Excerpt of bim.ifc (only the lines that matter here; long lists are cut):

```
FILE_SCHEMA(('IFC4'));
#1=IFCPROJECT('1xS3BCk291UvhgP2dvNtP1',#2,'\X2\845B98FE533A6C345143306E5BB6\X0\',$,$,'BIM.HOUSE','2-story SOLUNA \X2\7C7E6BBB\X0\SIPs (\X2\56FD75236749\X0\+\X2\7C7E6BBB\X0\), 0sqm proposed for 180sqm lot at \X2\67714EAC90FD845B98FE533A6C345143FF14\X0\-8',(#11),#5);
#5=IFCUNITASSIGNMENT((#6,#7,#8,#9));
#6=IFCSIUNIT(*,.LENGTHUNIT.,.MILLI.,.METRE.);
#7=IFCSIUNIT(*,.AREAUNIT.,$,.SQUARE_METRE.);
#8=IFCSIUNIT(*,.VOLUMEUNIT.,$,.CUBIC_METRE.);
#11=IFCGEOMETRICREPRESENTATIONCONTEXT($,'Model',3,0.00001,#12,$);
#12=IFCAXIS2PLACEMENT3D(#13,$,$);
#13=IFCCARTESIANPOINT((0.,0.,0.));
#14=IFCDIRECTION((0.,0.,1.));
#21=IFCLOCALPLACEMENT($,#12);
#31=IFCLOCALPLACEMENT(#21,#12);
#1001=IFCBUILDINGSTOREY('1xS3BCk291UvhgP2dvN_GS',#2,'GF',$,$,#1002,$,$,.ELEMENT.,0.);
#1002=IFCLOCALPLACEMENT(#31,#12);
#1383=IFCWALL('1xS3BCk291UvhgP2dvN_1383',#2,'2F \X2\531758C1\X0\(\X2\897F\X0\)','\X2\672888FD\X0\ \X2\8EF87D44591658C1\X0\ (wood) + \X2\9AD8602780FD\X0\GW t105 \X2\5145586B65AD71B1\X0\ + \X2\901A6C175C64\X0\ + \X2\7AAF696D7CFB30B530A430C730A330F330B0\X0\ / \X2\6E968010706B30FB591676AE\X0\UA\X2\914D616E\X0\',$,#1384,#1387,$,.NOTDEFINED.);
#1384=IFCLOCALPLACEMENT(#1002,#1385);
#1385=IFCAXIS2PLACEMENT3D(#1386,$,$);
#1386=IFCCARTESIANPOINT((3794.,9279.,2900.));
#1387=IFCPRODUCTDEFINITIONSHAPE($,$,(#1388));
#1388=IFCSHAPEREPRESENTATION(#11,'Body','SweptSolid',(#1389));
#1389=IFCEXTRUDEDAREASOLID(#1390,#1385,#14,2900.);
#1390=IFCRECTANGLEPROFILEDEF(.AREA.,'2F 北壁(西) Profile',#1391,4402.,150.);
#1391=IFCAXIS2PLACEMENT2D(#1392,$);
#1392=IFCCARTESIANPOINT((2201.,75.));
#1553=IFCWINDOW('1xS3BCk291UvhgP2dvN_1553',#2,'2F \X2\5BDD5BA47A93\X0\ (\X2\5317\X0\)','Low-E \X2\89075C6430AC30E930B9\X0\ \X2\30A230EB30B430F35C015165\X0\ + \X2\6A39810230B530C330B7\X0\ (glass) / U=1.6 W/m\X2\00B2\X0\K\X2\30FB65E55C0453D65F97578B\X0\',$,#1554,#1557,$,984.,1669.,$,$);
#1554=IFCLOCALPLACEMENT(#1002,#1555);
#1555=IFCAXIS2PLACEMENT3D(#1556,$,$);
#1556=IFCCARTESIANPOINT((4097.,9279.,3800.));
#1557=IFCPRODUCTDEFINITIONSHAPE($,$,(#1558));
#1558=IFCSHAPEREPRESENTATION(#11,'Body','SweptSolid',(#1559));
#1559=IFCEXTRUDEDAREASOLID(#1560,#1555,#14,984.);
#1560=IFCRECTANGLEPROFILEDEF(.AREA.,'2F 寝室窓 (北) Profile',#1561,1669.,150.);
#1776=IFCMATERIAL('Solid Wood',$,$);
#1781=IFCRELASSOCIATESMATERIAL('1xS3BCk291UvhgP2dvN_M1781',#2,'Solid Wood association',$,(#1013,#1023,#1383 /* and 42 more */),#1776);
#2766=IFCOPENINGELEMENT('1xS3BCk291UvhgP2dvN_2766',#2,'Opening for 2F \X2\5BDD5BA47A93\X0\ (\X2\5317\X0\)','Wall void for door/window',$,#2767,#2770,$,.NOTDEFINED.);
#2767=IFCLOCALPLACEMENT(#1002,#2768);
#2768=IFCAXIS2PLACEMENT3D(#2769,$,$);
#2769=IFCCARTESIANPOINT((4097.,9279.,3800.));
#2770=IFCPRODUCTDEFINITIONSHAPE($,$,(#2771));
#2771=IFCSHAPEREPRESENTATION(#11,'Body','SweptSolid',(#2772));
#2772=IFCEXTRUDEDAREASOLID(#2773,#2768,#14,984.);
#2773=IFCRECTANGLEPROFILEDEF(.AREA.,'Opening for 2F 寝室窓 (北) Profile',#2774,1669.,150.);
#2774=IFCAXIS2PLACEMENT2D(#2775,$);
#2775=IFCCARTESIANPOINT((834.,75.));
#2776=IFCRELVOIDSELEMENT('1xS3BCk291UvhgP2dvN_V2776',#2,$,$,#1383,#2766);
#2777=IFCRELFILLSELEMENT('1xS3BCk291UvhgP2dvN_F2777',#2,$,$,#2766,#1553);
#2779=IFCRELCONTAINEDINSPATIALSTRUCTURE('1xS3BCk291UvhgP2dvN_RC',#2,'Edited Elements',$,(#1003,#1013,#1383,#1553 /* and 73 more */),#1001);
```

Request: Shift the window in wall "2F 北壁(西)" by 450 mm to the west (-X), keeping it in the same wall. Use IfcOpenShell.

```python
import ifcopenshell
import ifcopenshell.api.geometry
import ifcopenshell.util.placement

model = ifcopenshell.open("bim.ifc")

window = model.by_guid("1xS3BCk291UvhgP2dvN_1553")
opening = window.FillsVoids[0].RelatingOpeningElement
wall = opening.VoidsElements[0].RelatingBuildingElement

wall_matrix = ifcopenshell.util.placement.get_local_placement(wall.ObjectPlacement)
shift = wall_matrix[:3, 0] * -450.0
before = ifcopenshell.util.placement.get_local_placement(window.ObjectPlacement)[:3, 3].copy()

# The window is not placed relative to its opening, so move both.
for product in (opening, window):
    matrix = ifcopenshell.util.placement.get_local_placement(product.ObjectPlacement)
    matrix[:3, 3] += shift
    ifcopenshell.api.geometry.edit_object_placement(model, product=product, matrix=matrix, is_si=False)

after = ifcopenshell.util.placement.get_local_placement(window.ObjectPlacement)[:3, 3]
print("window moved by", (after - before).round(3) + 0.0)

model.write("bim_updated.ifc")
```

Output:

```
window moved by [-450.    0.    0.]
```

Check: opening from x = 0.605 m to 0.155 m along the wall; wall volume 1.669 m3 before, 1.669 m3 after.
